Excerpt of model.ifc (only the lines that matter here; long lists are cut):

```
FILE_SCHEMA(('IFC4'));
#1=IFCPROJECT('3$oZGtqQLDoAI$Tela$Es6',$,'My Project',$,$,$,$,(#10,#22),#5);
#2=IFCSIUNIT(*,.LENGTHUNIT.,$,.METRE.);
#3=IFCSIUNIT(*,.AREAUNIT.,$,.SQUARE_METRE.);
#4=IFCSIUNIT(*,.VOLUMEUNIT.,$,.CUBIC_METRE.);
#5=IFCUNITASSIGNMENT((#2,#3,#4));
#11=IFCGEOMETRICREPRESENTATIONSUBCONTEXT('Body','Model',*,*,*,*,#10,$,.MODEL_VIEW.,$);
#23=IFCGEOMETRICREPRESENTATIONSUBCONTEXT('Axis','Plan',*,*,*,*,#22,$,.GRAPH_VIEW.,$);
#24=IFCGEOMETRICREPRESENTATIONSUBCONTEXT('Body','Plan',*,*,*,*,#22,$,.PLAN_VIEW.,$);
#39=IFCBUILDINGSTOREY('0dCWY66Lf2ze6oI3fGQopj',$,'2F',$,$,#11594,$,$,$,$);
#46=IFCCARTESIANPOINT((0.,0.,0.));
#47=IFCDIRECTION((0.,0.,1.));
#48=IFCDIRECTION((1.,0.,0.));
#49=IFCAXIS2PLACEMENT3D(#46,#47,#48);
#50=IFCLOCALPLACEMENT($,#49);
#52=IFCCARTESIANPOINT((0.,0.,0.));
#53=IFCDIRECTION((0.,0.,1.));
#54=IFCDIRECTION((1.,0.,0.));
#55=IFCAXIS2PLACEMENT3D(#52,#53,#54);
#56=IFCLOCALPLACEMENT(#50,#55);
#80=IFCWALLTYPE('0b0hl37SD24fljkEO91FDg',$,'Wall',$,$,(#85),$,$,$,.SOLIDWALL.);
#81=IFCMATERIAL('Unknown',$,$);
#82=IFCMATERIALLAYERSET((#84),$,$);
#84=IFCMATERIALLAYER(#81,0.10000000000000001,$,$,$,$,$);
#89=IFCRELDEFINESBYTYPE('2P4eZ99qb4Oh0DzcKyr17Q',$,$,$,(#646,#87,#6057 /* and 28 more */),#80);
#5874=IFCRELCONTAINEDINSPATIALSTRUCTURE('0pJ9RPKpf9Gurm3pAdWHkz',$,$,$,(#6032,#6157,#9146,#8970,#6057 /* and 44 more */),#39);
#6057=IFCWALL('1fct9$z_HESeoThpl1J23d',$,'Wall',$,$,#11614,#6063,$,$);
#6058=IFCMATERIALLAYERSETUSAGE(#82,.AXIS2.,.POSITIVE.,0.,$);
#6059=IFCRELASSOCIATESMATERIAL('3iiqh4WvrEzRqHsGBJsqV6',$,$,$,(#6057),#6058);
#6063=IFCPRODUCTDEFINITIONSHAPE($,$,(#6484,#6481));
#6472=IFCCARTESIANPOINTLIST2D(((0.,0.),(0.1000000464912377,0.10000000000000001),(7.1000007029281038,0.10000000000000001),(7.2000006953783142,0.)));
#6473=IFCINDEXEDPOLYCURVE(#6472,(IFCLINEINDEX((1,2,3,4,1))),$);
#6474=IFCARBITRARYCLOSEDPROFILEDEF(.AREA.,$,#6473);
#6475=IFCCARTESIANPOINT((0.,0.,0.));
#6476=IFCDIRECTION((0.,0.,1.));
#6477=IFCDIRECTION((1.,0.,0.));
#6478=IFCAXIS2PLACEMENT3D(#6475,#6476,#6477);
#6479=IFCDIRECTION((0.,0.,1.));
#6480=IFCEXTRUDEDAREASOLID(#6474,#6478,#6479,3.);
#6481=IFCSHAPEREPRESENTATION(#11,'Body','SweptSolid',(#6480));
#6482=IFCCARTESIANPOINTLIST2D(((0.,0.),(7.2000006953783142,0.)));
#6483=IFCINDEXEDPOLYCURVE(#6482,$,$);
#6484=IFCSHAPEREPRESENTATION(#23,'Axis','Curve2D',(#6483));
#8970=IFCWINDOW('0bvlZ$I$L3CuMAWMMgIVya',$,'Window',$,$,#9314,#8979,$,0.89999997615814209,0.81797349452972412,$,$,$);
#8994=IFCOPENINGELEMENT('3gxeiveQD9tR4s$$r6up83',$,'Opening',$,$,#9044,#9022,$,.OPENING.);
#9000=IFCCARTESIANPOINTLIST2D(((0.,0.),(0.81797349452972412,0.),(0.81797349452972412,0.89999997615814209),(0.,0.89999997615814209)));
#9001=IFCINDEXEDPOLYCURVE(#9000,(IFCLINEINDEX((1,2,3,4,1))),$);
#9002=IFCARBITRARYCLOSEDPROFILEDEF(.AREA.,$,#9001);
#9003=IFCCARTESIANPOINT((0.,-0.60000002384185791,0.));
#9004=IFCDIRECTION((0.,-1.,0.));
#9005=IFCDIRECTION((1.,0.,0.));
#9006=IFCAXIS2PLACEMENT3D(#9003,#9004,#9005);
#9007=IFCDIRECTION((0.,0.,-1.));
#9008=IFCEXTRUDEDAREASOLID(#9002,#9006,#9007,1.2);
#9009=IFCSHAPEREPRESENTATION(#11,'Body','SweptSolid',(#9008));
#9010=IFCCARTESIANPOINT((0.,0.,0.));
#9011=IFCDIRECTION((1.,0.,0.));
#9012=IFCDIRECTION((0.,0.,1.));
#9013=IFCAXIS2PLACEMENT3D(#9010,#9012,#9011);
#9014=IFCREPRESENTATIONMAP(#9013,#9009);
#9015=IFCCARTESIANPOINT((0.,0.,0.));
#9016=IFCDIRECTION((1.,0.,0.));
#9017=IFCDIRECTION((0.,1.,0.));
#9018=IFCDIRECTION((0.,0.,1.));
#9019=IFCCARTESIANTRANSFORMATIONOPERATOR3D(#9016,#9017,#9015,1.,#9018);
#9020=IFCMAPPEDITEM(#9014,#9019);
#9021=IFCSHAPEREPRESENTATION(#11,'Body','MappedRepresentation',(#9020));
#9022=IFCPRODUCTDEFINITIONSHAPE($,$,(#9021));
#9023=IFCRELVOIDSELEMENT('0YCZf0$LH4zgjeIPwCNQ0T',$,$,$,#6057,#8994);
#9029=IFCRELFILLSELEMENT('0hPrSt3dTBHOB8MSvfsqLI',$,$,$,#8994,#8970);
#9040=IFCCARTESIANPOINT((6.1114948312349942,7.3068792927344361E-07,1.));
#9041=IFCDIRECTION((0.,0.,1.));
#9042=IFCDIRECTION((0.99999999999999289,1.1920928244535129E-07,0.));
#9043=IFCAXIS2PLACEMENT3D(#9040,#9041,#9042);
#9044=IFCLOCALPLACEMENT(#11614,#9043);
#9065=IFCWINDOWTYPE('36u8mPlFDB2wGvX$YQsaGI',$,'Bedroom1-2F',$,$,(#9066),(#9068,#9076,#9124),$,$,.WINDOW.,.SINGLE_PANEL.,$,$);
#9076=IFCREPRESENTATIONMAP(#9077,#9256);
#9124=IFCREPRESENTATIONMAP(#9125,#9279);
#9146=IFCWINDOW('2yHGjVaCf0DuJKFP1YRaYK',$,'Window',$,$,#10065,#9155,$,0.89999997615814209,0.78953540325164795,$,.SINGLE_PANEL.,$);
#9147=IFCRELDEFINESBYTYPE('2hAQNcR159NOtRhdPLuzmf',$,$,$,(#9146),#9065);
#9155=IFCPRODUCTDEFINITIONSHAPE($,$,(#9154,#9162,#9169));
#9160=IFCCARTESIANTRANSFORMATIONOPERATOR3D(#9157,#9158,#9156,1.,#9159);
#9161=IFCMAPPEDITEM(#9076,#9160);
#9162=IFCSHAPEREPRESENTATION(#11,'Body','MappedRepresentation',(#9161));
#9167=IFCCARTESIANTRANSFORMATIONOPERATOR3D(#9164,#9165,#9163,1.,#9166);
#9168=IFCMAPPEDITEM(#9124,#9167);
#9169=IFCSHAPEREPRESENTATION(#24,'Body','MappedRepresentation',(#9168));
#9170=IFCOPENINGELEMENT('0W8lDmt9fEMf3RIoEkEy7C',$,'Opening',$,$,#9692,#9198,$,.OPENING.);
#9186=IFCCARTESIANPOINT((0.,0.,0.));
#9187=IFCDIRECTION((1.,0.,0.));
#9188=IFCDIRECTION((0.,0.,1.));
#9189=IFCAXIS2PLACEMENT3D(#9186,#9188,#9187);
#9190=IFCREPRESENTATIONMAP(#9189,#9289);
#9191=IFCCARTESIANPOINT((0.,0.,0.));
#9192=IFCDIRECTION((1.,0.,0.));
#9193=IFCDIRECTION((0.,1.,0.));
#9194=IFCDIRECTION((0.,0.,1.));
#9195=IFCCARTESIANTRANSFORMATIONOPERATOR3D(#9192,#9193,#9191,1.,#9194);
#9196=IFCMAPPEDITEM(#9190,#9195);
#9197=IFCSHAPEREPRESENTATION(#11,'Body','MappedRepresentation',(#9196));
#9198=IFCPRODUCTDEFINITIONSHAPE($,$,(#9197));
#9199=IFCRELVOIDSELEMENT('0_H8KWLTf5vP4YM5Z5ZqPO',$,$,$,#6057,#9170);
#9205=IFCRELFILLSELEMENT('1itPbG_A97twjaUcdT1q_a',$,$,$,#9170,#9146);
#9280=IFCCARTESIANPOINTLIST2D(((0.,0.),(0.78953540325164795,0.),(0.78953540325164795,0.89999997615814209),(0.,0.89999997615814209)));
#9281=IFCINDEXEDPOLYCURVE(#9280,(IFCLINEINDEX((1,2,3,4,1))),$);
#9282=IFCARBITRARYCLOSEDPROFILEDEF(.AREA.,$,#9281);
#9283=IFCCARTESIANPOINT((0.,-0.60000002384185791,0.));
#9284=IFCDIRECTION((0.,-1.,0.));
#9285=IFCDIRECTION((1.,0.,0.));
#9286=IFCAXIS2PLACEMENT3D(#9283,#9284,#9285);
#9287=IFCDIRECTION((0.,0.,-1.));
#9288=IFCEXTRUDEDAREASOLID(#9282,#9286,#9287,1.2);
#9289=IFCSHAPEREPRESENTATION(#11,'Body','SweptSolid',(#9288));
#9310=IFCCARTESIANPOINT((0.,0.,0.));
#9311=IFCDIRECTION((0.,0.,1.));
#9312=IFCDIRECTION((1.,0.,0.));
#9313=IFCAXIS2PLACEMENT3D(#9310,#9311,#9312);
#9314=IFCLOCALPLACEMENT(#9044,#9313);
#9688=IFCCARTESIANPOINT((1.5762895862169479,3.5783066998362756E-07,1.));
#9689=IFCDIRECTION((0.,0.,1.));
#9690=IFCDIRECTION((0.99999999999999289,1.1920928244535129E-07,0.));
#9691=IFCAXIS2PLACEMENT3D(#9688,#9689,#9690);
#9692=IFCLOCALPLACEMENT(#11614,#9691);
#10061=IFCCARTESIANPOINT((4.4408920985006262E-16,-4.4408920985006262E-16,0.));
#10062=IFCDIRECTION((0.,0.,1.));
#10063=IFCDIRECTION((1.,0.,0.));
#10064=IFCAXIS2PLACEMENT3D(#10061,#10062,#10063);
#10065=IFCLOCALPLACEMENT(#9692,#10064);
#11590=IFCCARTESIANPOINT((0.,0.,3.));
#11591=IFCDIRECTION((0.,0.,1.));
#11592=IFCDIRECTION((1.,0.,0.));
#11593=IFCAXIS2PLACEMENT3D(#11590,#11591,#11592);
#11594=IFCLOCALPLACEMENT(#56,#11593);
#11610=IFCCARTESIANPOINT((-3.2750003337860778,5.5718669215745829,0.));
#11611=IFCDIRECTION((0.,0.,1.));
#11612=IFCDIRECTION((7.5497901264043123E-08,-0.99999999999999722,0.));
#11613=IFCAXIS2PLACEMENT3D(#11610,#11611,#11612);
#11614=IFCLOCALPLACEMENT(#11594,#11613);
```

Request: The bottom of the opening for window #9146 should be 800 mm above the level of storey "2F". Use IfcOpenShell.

```python
import numpy as np
import ifcopenshell
import ifcopenshell.api.geometry
import ifcopenshell.geom
import ifcopenshell.util.element
import ifcopenshell.util.placement
import ifcopenshell.util.shape
import ifcopenshell.util.unit

model = ifcopenshell.open("model.ifc")
unit_scale = ifcopenshell.util.unit.calculate_unit_scale(model)

window = model.by_guid("2yHGjVaCf0DuJKFP1YRaYK")
opening = window.FillsVoids[0].RelatingOpeningElement
storey = ifcopenshell.util.element.get_container(window, ifc_class="IfcBuildingStorey")
level = ifcopenshell.util.placement.get_local_placement(storey.ObjectPlacement)[2, 3]

# The opening's origin need not be at the sill, so measure its lowest point.
shape = ifcopenshell.geom.create_shape(ifcopenshell.geom.settings(), opening)
bottom = ifcopenshell.util.shape.get_shape_bottom_elevation(shape, shape.geometry) / unit_scale
dz = level + 0.8 / unit_scale - bottom

shift = np.array([0.0, 0.0, dz])
# The window is placed relative to its opening, so it follows when the opening moves.
matrix = ifcopenshell.util.placement.get_local_placement(opening.ObjectPlacement)
matrix[:3, 3] += shift
ifcopenshell.api.geometry.edit_object_placement(
    model, product=opening, matrix=matrix, is_si=False, should_transform_children=True
)

print(f"moved by {dz * unit_scale:+.3f} m")

model.write("model_v2.ifc")
```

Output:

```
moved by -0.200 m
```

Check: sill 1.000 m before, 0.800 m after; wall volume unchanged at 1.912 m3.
